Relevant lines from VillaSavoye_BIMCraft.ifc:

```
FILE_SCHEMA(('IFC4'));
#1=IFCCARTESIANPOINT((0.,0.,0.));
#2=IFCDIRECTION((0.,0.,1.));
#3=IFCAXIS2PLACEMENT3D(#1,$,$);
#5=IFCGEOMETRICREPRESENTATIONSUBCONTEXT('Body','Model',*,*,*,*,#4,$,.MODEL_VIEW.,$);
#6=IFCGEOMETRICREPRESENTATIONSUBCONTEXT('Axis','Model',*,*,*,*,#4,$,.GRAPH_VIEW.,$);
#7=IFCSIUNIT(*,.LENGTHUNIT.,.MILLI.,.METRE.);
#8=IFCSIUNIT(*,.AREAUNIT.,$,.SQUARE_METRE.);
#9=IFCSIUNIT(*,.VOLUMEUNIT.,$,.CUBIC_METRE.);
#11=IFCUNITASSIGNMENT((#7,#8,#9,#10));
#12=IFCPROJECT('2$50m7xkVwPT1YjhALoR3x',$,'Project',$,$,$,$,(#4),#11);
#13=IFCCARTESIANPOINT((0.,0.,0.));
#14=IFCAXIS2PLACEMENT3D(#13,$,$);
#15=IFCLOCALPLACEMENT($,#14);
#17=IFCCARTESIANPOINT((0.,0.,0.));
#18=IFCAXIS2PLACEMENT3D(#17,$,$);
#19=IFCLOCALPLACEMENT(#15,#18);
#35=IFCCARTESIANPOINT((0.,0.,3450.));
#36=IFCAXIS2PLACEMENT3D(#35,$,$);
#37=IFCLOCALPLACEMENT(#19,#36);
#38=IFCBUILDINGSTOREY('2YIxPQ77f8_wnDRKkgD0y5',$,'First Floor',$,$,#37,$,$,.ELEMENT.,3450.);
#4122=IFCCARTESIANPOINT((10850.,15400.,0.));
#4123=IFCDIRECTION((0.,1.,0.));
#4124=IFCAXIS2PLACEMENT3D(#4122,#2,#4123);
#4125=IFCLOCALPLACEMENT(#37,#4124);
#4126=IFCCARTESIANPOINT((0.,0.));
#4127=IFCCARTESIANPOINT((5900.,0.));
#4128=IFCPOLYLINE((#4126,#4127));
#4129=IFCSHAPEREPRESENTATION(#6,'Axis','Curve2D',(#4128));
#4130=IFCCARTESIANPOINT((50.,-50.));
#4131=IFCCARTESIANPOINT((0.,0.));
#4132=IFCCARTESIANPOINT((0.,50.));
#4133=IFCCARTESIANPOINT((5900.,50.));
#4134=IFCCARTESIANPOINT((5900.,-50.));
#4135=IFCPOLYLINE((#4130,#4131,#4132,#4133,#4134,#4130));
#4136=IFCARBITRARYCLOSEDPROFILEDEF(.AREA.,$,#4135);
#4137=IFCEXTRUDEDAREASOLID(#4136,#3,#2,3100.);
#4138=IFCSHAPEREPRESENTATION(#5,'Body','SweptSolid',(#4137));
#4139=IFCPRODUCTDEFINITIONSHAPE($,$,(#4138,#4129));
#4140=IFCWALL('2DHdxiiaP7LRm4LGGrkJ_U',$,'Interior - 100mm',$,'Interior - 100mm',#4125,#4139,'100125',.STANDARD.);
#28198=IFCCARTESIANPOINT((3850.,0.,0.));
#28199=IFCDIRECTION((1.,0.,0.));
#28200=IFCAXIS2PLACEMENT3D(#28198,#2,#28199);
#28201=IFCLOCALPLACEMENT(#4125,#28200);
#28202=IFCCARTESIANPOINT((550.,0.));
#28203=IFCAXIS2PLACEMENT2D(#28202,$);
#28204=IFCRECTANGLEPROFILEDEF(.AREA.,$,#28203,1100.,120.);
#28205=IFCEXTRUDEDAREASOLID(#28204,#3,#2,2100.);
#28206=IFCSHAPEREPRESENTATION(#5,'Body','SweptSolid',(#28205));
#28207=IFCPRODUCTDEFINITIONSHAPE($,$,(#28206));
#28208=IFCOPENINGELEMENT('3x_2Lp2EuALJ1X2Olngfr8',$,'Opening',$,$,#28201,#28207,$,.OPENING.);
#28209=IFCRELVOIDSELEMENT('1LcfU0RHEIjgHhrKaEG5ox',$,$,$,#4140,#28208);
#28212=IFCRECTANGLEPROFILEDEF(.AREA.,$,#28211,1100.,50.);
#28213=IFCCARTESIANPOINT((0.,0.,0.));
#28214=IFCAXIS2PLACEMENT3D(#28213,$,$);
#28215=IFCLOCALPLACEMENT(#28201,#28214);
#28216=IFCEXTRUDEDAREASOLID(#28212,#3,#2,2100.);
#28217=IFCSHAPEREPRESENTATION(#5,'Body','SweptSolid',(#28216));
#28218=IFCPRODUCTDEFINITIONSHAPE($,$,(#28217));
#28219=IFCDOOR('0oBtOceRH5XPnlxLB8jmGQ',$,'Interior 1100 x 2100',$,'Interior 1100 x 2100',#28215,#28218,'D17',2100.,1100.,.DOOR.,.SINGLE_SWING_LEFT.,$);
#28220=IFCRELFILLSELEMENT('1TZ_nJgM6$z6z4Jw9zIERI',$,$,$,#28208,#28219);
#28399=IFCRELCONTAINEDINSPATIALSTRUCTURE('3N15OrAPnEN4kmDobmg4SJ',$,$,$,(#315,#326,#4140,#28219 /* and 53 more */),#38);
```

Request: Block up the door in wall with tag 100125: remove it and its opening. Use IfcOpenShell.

```python
import ifcopenshell
import ifcopenshell.api.feature
import ifcopenshell.api.root
import ifcopenshell.geom
import ifcopenshell.util.shape

model = ifcopenshell.open("VillaSavoye_BIMCraft.ifc")
settings = ifcopenshell.geom.settings()


def volume(element):
    """Net volume in cubic metres, openings subtracted."""
    shape = ifcopenshell.geom.create_shape(settings, element)
    return ifcopenshell.util.shape.get_volume(shape.geometry)


door = model.by_id(28219)
opening = door.FillsVoids[0].RelatingOpeningElement
wall = opening.VoidsElements[0].RelatingBuildingElement
before = volume(wall)

ifcopenshell.api.root.remove_product(model, product=door)
ifcopenshell.api.feature.remove_feature(model, feature=opening)

after = volume(wall)

print(f"wall volume {before:.3f} -> {after:.3f} m3")

model.write("VillaSavoye_BIMCraft-out.ifc")
```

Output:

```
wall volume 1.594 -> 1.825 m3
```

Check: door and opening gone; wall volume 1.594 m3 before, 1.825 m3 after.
